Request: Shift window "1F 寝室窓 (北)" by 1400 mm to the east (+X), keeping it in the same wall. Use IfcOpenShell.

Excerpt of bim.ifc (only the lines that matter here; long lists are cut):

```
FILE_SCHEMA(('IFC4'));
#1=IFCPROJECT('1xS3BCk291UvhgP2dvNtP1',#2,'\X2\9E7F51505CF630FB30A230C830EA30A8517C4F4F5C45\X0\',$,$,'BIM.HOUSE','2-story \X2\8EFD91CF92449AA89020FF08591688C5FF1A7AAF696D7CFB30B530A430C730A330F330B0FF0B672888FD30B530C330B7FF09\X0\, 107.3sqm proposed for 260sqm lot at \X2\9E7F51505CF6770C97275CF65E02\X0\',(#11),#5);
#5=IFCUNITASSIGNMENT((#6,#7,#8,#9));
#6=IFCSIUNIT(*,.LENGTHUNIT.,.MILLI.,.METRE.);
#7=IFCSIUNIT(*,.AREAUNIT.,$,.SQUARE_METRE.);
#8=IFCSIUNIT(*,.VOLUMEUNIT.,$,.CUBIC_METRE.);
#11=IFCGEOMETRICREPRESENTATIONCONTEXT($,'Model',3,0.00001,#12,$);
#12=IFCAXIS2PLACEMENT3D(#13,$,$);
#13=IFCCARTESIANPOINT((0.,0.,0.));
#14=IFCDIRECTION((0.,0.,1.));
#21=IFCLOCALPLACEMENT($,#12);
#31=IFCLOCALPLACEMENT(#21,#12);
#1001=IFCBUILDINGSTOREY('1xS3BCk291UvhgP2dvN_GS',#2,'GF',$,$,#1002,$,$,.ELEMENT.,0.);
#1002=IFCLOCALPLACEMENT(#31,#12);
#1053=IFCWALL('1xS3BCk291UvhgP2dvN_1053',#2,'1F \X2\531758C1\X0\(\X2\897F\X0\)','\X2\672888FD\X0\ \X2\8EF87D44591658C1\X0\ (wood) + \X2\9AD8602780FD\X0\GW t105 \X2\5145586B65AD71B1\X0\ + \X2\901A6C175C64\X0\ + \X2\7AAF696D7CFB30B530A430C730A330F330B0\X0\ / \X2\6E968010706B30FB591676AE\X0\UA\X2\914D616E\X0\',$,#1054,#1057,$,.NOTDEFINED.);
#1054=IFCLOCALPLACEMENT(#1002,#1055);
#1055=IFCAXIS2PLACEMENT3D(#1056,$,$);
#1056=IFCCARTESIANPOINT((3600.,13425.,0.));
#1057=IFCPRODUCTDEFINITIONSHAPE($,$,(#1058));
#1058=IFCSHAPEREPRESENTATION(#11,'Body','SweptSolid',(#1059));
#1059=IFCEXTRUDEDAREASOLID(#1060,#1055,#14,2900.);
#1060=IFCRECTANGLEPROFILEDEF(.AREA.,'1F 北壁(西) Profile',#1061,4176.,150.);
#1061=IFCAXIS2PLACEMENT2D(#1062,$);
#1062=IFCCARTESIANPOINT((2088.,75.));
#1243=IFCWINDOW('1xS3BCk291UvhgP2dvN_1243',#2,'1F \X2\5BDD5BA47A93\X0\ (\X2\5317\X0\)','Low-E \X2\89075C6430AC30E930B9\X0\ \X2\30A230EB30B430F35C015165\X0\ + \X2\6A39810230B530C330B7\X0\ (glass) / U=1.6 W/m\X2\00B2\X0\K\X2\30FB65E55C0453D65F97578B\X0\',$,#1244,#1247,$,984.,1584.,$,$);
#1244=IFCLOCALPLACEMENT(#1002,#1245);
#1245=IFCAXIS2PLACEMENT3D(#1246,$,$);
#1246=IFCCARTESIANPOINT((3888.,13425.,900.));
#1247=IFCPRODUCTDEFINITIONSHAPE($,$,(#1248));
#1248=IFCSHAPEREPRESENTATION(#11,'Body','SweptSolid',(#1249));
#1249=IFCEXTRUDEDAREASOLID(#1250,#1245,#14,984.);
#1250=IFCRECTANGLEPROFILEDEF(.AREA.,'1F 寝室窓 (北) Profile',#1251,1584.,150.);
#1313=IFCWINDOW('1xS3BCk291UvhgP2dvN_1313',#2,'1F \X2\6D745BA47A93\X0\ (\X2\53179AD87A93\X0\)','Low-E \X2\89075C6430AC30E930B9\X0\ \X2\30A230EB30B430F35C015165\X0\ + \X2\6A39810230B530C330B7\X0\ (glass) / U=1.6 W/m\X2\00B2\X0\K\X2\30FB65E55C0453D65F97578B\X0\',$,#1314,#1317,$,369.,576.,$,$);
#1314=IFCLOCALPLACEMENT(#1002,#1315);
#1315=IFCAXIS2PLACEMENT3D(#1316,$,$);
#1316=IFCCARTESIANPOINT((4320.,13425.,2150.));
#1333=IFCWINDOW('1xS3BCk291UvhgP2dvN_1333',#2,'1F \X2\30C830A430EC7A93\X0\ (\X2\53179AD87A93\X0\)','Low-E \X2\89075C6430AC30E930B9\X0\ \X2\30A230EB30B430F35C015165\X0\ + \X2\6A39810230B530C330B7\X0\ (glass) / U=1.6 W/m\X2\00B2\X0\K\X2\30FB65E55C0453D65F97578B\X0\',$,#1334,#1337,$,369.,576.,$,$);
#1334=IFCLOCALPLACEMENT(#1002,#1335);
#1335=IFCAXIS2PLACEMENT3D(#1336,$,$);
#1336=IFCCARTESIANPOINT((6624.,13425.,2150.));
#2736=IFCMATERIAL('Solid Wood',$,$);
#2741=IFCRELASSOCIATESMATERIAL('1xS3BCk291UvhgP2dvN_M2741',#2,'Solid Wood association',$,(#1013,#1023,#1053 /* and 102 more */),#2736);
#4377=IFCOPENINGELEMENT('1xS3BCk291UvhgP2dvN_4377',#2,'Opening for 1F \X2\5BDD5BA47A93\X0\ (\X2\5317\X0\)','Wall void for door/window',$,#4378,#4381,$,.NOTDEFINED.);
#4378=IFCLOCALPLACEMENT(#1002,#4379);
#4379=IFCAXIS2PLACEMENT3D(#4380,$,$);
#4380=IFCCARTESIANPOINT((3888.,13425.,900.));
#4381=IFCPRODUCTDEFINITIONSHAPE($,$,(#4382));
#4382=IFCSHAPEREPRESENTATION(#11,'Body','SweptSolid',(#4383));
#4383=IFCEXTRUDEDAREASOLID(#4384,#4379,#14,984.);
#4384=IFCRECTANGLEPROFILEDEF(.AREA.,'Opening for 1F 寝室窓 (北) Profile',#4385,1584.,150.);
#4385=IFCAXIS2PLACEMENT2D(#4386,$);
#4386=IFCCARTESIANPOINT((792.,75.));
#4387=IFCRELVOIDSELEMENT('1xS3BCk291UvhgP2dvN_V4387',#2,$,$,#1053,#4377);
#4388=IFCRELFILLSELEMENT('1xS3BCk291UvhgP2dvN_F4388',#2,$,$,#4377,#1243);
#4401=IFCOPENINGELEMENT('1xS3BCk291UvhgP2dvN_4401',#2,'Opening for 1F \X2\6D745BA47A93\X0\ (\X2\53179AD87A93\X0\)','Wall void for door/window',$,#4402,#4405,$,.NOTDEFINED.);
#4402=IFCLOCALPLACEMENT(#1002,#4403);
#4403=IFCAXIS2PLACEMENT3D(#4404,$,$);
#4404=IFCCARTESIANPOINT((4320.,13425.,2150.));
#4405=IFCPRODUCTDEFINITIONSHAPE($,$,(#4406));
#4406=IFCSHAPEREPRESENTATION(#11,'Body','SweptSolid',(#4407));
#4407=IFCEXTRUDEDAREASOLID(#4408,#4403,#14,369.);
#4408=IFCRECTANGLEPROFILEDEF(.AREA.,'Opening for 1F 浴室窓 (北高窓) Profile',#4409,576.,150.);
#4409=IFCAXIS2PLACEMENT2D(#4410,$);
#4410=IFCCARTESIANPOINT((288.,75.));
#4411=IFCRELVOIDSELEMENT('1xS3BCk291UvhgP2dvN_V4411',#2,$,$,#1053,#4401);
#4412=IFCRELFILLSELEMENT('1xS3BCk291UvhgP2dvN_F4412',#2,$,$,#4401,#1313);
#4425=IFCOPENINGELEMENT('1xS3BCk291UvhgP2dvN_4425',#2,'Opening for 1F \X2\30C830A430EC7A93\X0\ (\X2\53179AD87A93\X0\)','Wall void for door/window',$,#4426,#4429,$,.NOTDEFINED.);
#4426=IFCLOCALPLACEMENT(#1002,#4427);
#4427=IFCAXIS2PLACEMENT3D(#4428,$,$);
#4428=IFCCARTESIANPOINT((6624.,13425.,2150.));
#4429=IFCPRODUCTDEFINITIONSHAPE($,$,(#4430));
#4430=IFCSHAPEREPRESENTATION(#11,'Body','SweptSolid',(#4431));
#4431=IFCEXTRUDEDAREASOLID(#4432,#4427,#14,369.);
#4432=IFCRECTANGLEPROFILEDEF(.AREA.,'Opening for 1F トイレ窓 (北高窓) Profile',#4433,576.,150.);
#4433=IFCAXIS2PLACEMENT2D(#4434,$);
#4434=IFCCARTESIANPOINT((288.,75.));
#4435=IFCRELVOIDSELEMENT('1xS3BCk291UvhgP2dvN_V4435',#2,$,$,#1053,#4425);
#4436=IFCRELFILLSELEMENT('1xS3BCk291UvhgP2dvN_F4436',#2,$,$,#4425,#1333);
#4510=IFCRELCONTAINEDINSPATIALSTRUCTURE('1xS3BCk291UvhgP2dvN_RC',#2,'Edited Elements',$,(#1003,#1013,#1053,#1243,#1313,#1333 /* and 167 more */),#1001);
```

```python
import ifcopenshell
import ifcopenshell.api.geometry
import ifcopenshell.util.placement
import ifcopenshell.util.unit

model = ifcopenshell.open("bim.ifc")
unit_scale = ifcopenshell.util.unit.calculate_unit_scale(model)

window = model.by_guid("1xS3BCk291UvhgP2dvN_1243")
opening = window.FillsVoids[0].RelatingOpeningElement
wall = opening.VoidsElements[0].RelatingBuildingElement

wall_matrix = ifcopenshell.util.placement.get_local_placement(wall.ObjectPlacement)
shift = wall_matrix[:3, 0] * 1.4 / unit_scale
before = ifcopenshell.util.placement.get_local_placement(window.ObjectPlacement)[:3, 3].copy()

# The window is not placed relative to its opening, so move both.
for product in (opening, window):
    matrix = ifcopenshell.util.placement.get_local_placement(product.ObjectPlacement)
    matrix[:3, 3] += shift
    ifcopenshell.api.geometry.edit_object_placement(model, product=product, matrix=matrix, is_si=False)

after = ifcopenshell.util.placement.get_local_placement(window.ObjectPlacement)[:3, 3]
print("window moved by", (after - before).round(3) + 0.0)

model.write("bim_v2.ifc")
```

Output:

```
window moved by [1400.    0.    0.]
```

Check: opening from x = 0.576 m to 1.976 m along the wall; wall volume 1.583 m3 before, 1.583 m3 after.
